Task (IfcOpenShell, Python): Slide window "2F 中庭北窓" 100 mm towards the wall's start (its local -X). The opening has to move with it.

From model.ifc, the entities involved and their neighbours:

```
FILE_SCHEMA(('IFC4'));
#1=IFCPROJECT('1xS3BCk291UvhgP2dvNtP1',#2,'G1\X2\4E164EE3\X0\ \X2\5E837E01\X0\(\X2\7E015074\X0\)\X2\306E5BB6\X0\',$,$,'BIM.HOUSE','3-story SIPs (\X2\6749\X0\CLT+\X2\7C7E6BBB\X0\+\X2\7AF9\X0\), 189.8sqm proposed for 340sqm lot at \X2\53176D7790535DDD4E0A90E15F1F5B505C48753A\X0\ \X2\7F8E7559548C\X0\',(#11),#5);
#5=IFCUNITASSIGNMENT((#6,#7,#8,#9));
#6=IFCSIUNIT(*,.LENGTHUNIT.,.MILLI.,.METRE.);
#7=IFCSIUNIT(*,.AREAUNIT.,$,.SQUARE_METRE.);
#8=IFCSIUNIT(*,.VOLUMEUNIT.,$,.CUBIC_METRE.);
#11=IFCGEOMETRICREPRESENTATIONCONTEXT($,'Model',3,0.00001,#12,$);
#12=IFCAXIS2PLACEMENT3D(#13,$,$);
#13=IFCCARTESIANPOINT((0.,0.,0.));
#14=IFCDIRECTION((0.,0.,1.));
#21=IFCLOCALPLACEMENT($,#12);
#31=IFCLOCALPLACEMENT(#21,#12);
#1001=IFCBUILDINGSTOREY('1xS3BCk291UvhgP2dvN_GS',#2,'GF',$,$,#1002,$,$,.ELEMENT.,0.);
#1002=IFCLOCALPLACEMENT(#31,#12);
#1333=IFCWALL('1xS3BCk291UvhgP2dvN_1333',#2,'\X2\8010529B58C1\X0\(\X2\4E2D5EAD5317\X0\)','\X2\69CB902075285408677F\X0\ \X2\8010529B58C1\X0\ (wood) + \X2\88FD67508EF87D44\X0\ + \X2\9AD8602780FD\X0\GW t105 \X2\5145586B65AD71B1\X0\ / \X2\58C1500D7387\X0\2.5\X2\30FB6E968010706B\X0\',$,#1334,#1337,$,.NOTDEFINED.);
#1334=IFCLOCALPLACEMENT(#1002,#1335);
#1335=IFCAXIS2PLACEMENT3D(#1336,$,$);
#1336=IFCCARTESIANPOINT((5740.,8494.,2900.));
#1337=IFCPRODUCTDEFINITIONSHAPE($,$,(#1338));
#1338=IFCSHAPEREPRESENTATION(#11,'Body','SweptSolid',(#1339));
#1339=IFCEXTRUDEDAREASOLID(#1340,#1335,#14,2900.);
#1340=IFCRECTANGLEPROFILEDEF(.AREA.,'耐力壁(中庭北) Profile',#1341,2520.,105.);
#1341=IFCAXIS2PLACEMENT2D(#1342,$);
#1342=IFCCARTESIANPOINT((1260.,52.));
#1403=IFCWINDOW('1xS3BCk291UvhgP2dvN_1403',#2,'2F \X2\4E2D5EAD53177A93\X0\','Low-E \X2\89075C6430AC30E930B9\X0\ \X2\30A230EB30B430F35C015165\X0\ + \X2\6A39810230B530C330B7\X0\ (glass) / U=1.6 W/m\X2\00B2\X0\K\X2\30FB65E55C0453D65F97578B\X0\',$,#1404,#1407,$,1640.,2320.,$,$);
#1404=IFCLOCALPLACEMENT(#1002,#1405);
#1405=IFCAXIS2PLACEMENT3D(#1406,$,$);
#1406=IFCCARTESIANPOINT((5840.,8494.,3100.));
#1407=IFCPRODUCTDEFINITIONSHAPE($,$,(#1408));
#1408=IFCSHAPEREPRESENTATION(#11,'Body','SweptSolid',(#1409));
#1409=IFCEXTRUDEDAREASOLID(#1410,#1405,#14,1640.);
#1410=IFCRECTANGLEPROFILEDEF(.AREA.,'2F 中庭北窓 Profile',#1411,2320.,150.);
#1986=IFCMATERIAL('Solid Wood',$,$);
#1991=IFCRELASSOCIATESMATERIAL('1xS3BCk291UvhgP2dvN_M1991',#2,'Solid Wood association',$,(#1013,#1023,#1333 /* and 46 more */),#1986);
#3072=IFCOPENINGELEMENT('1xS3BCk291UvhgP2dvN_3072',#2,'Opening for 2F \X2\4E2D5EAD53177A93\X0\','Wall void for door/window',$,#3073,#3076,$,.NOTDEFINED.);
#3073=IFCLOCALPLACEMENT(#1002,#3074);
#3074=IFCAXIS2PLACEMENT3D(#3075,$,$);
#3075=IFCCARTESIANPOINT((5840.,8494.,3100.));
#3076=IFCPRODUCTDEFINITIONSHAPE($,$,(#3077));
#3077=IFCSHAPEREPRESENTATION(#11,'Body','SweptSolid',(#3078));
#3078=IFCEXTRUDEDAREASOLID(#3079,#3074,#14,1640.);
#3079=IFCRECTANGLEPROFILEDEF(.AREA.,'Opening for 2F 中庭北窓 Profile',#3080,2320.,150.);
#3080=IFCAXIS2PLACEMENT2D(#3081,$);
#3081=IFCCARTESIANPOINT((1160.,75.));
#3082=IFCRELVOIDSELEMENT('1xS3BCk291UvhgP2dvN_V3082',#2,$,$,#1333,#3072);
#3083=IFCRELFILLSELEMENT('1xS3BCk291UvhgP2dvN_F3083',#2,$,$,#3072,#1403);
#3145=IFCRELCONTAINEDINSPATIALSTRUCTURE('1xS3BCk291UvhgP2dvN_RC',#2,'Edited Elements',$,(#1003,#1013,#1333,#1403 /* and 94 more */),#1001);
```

```python
import ifcopenshell
import ifcopenshell.api.geometry
import ifcopenshell.util.placement
import ifcopenshell.util.unit

model = ifcopenshell.open("model.ifc")
unit_scale = ifcopenshell.util.unit.calculate_unit_scale(model)

window = model.by_guid("1xS3BCk291UvhgP2dvN_1403")
opening = window.FillsVoids[0].RelatingOpeningElement
wall = opening.VoidsElements[0].RelatingBuildingElement

wall_matrix = ifcopenshell.util.placement.get_local_placement(wall.ObjectPlacement)
shift = wall_matrix[:3, 0] * -0.1 / unit_scale
before = ifcopenshell.util.placement.get_local_placement(window.ObjectPlacement)[:3, 3].copy()

# The window is not placed relative to its opening, so move both.
for product in (opening, window):
    matrix = ifcopenshell.util.placement.get_local_placement(product.ObjectPlacement)
    matrix[:3, 3] += shift
    ifcopenshell.api.geometry.edit_object_placement(model, product=product, matrix=matrix, is_si=False)

after = ifcopenshell.util.placement.get_local_placement(window.ObjectPlacement)[:3, 3]
print("window moved by", (after - before).round(3) + 0.0)

model.write("model_edited.ifc")
```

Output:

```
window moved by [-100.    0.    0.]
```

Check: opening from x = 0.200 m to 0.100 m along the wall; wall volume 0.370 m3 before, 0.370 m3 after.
